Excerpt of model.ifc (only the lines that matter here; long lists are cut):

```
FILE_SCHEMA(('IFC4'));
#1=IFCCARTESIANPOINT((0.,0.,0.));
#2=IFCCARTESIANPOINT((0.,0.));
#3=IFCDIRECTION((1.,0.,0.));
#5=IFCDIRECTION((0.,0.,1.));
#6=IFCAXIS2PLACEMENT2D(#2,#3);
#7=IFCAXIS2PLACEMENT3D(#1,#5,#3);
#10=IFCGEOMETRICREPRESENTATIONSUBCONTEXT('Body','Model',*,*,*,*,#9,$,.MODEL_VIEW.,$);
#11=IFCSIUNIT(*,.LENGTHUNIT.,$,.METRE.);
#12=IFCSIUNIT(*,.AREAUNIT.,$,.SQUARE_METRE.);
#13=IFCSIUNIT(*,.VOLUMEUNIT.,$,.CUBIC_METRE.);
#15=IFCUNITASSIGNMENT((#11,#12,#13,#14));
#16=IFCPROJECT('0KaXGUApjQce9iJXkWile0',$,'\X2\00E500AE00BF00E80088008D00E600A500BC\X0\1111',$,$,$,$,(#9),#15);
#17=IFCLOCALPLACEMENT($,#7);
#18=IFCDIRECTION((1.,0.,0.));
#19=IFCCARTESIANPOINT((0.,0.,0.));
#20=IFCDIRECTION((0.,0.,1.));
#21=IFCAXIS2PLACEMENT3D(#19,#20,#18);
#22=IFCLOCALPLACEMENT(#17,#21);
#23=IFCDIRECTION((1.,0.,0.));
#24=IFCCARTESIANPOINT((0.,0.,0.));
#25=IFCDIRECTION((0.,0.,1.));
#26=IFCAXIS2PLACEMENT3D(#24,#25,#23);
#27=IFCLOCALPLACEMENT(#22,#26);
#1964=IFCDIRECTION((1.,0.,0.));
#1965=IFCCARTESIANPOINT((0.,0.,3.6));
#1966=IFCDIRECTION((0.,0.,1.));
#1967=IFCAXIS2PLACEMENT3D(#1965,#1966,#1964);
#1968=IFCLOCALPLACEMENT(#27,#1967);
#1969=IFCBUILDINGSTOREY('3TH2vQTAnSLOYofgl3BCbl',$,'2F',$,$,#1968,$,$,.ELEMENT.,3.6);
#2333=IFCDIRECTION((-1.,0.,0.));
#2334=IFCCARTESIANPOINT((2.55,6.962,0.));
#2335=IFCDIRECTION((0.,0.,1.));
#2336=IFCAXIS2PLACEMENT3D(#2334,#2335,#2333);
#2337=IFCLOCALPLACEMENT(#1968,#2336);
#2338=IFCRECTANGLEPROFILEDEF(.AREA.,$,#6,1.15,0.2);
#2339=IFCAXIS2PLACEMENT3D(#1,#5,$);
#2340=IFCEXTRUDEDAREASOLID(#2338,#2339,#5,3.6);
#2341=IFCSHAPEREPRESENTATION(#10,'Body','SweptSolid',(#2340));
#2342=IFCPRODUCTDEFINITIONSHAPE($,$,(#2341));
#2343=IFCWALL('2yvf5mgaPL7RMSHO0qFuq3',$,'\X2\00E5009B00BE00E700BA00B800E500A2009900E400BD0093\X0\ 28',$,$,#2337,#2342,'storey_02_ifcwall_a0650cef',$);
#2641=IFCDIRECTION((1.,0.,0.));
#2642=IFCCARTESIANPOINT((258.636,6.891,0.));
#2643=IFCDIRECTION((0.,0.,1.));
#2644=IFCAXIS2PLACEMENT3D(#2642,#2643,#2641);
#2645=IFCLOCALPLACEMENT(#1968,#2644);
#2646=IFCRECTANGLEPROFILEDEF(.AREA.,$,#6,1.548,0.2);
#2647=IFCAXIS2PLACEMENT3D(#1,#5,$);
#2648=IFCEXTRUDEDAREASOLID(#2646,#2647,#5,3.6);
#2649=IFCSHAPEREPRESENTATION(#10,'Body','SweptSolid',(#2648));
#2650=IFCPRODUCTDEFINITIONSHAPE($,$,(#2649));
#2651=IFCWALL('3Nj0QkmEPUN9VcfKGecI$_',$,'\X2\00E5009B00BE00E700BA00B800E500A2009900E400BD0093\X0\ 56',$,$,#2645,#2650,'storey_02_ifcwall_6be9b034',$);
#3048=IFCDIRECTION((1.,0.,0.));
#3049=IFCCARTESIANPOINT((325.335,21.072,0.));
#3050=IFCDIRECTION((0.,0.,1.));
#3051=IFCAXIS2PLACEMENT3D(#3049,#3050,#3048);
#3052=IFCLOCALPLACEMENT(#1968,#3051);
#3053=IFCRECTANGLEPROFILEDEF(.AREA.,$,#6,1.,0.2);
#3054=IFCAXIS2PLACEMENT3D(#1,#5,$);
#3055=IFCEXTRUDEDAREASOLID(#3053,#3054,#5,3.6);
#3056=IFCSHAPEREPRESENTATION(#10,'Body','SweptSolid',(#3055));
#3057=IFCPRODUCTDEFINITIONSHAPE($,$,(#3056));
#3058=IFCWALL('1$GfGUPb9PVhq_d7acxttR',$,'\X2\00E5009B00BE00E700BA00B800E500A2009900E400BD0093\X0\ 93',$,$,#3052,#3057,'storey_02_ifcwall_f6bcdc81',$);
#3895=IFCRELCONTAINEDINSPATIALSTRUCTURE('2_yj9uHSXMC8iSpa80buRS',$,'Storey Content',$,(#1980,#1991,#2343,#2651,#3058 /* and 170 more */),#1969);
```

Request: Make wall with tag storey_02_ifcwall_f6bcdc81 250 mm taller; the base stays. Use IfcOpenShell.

```python
import ifcopenshell
import ifcopenshell.geom
import ifcopenshell.util.representation
import ifcopenshell.util.shape

model = ifcopenshell.open("model.ifc")
settings = ifcopenshell.geom.settings()


def volume(element):
    """Net volume in cubic metres, openings subtracted."""
    shape = ifcopenshell.geom.create_shape(settings, element)
    return ifcopenshell.util.shape.get_volume(shape.geometry)


wall = model.by_guid("1$GfGUPb9PVhq_d7acxttR")
before = volume(wall)

body = ifcopenshell.util.representation.get_representation(wall, "Model", "Body")
solid = body.Items[0]
old_height = solid.Depth
solid.Depth += 0.25
after = volume(wall)

print(f"height {old_height:g} -> {solid.Depth:g}, volume {before:.3f} -> {after:.3f} m3")

model.write("model_updated.ifc")
```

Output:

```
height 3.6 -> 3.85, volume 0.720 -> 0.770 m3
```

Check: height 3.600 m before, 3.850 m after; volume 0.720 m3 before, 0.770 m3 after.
